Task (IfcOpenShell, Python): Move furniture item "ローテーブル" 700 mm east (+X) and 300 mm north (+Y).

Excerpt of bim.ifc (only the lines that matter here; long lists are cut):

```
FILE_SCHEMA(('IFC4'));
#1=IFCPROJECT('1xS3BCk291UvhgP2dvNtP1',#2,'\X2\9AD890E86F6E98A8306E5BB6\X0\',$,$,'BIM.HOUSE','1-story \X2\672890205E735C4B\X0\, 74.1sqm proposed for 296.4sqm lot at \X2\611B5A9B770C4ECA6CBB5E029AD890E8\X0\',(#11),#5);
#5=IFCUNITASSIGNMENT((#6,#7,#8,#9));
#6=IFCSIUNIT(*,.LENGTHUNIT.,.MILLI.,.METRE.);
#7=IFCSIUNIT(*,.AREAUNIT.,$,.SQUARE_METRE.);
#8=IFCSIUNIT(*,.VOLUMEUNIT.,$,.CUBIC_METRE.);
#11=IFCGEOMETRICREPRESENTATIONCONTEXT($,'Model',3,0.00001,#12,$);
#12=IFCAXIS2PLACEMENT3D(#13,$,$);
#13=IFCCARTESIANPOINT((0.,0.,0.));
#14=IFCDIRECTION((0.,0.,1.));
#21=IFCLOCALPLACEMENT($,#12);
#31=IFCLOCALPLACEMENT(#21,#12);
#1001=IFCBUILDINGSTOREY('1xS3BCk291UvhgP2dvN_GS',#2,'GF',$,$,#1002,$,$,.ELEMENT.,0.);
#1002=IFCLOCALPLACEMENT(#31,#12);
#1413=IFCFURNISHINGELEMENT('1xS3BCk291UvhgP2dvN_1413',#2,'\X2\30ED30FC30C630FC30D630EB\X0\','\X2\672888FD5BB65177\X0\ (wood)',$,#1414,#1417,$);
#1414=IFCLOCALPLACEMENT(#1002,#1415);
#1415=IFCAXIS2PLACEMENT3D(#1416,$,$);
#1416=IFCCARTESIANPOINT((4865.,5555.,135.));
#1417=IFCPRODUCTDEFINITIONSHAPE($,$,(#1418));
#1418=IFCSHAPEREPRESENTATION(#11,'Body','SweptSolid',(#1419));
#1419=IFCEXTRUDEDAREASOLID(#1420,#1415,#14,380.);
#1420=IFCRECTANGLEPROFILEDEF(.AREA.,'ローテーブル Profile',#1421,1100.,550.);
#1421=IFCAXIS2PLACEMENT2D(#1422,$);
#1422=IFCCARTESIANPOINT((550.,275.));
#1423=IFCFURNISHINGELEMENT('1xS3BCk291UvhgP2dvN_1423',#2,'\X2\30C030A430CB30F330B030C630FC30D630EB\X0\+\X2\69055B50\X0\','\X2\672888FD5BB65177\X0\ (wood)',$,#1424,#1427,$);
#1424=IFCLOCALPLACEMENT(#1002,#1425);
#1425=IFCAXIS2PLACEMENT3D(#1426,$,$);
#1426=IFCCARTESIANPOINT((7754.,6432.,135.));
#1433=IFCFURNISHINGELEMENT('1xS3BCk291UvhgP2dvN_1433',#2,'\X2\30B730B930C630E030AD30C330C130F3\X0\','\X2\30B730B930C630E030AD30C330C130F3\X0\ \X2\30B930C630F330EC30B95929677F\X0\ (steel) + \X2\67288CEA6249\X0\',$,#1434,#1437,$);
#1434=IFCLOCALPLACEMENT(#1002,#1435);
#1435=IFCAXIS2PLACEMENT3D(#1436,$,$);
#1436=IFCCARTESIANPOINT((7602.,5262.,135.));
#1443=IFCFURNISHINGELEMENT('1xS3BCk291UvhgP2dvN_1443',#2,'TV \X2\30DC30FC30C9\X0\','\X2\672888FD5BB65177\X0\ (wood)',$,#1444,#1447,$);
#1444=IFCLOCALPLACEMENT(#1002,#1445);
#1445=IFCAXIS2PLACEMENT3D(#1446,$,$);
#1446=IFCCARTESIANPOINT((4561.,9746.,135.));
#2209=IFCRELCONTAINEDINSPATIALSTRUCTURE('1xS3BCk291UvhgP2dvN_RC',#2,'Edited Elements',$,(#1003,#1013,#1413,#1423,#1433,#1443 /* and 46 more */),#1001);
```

```python
import ifcopenshell
import ifcopenshell.api.geometry
import ifcopenshell.util.placement

model = ifcopenshell.open("bim.ifc")

item = model.by_guid("1xS3BCk291UvhgP2dvN_1413")
matrix = ifcopenshell.util.placement.get_local_placement(item.ObjectPlacement)
matrix[0, 3] += 700.0
matrix[1, 3] += 300.0
ifcopenshell.api.geometry.edit_object_placement(model, product=item, matrix=matrix, is_si=False)

print(ifcopenshell.util.placement.get_local_placement(item.ObjectPlacement).round(3) + 0.0)

model.write("bim_updated.ifc")
```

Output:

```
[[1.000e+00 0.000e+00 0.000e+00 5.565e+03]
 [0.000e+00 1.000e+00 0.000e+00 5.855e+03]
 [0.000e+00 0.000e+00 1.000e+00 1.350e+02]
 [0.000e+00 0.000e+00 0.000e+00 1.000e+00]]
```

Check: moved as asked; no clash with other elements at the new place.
